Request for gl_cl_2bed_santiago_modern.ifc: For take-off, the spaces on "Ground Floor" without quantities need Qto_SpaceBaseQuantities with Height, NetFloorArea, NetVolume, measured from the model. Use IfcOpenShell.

First a look at what the model holds.

```python
import ifcopenshell
import ifcopenshell.util.element
import ifcopenshell.util.unit

model = ifcopenshell.open("gl_cl_2bed_santiago_modern.ifc")
print(model.schema)
for unit_type in ("LENGTHUNIT", "AREAUNIT", "VOLUMEUNIT"):
    print(unit_type, ifcopenshell.util.unit.calculate_unit_scale(model, unit_type))
storey = next(s for s in model.by_type("IfcBuildingStorey") if s.Name == "Ground Floor")
spaces = [e for e in ifcopenshell.util.element.get_decomposition(storey) if e.is_a("IfcSpace")]
for e in sorted(spaces, key=lambda e: e.id()):
    print(e.id(), e.is_a(), e.Name, list(ifcopenshell.util.element.get_psets(e, qtos_only=True)), sep=" | ")
```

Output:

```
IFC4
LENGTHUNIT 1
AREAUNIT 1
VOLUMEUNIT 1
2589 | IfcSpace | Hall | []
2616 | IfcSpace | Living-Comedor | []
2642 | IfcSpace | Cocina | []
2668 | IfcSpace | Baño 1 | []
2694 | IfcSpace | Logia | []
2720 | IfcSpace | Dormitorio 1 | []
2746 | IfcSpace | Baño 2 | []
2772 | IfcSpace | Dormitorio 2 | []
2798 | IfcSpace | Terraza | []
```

```python
import ifcopenshell
import ifcopenshell.api.pset
import ifcopenshell.geom
import ifcopenshell.util.element
import ifcopenshell.util.shape
import ifcopenshell.util.unit

model = ifcopenshell.open("gl_cl_2bed_santiago_modern.ifc")
unit_scale = ifcopenshell.util.unit.calculate_unit_scale(model)
area_scale = ifcopenshell.util.unit.calculate_unit_scale(model, "AREAUNIT")
volume_scale = ifcopenshell.util.unit.calculate_unit_scale(model, "VOLUMEUNIT")
settings = ifcopenshell.geom.settings()

storey = next(s for s in model.by_type("IfcBuildingStorey") if s.Name == "Ground Floor")
spaces = [e for e in ifcopenshell.util.element.get_decomposition(storey) if e.is_a("IfcSpace")]

for e in sorted(spaces, key=lambda e: e.id()):
    if ifcopenshell.util.element.get_psets(e, qtos_only=True, should_inherit=False):
        continue
    # Geometry comes back in metres, in the element's own axes.
    shape = ifcopenshell.geom.create_shape(settings, e)
    values = {
        "Height": ifcopenshell.util.shape.get_z(shape.geometry) / unit_scale,
        "NetFloorArea": ifcopenshell.util.shape.get_footprint_area(shape.geometry) / area_scale,
        "NetVolume": ifcopenshell.util.shape.get_volume(shape.geometry) / volume_scale,
    }
    qto = ifcopenshell.api.pset.add_qto(model, product=e, name="Qto_SpaceBaseQuantities")
    ifcopenshell.api.pset.edit_qto(model, qto=qto, properties=values)
    print(e.id(), {k: round(v, 3) for k, v in values.items()})

model.write("gl_cl_2bed_santiago_modern_updated.ifc")
```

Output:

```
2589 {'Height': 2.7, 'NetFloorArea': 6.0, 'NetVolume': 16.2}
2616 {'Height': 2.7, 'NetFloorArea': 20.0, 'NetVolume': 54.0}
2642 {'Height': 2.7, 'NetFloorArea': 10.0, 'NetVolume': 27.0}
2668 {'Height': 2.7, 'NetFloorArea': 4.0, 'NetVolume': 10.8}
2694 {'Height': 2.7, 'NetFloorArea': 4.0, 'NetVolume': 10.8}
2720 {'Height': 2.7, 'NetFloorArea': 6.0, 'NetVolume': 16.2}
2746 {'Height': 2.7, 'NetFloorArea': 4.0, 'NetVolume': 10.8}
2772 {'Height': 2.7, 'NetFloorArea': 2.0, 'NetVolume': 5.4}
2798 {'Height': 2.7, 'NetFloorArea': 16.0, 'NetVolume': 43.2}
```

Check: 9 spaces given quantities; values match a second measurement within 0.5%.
